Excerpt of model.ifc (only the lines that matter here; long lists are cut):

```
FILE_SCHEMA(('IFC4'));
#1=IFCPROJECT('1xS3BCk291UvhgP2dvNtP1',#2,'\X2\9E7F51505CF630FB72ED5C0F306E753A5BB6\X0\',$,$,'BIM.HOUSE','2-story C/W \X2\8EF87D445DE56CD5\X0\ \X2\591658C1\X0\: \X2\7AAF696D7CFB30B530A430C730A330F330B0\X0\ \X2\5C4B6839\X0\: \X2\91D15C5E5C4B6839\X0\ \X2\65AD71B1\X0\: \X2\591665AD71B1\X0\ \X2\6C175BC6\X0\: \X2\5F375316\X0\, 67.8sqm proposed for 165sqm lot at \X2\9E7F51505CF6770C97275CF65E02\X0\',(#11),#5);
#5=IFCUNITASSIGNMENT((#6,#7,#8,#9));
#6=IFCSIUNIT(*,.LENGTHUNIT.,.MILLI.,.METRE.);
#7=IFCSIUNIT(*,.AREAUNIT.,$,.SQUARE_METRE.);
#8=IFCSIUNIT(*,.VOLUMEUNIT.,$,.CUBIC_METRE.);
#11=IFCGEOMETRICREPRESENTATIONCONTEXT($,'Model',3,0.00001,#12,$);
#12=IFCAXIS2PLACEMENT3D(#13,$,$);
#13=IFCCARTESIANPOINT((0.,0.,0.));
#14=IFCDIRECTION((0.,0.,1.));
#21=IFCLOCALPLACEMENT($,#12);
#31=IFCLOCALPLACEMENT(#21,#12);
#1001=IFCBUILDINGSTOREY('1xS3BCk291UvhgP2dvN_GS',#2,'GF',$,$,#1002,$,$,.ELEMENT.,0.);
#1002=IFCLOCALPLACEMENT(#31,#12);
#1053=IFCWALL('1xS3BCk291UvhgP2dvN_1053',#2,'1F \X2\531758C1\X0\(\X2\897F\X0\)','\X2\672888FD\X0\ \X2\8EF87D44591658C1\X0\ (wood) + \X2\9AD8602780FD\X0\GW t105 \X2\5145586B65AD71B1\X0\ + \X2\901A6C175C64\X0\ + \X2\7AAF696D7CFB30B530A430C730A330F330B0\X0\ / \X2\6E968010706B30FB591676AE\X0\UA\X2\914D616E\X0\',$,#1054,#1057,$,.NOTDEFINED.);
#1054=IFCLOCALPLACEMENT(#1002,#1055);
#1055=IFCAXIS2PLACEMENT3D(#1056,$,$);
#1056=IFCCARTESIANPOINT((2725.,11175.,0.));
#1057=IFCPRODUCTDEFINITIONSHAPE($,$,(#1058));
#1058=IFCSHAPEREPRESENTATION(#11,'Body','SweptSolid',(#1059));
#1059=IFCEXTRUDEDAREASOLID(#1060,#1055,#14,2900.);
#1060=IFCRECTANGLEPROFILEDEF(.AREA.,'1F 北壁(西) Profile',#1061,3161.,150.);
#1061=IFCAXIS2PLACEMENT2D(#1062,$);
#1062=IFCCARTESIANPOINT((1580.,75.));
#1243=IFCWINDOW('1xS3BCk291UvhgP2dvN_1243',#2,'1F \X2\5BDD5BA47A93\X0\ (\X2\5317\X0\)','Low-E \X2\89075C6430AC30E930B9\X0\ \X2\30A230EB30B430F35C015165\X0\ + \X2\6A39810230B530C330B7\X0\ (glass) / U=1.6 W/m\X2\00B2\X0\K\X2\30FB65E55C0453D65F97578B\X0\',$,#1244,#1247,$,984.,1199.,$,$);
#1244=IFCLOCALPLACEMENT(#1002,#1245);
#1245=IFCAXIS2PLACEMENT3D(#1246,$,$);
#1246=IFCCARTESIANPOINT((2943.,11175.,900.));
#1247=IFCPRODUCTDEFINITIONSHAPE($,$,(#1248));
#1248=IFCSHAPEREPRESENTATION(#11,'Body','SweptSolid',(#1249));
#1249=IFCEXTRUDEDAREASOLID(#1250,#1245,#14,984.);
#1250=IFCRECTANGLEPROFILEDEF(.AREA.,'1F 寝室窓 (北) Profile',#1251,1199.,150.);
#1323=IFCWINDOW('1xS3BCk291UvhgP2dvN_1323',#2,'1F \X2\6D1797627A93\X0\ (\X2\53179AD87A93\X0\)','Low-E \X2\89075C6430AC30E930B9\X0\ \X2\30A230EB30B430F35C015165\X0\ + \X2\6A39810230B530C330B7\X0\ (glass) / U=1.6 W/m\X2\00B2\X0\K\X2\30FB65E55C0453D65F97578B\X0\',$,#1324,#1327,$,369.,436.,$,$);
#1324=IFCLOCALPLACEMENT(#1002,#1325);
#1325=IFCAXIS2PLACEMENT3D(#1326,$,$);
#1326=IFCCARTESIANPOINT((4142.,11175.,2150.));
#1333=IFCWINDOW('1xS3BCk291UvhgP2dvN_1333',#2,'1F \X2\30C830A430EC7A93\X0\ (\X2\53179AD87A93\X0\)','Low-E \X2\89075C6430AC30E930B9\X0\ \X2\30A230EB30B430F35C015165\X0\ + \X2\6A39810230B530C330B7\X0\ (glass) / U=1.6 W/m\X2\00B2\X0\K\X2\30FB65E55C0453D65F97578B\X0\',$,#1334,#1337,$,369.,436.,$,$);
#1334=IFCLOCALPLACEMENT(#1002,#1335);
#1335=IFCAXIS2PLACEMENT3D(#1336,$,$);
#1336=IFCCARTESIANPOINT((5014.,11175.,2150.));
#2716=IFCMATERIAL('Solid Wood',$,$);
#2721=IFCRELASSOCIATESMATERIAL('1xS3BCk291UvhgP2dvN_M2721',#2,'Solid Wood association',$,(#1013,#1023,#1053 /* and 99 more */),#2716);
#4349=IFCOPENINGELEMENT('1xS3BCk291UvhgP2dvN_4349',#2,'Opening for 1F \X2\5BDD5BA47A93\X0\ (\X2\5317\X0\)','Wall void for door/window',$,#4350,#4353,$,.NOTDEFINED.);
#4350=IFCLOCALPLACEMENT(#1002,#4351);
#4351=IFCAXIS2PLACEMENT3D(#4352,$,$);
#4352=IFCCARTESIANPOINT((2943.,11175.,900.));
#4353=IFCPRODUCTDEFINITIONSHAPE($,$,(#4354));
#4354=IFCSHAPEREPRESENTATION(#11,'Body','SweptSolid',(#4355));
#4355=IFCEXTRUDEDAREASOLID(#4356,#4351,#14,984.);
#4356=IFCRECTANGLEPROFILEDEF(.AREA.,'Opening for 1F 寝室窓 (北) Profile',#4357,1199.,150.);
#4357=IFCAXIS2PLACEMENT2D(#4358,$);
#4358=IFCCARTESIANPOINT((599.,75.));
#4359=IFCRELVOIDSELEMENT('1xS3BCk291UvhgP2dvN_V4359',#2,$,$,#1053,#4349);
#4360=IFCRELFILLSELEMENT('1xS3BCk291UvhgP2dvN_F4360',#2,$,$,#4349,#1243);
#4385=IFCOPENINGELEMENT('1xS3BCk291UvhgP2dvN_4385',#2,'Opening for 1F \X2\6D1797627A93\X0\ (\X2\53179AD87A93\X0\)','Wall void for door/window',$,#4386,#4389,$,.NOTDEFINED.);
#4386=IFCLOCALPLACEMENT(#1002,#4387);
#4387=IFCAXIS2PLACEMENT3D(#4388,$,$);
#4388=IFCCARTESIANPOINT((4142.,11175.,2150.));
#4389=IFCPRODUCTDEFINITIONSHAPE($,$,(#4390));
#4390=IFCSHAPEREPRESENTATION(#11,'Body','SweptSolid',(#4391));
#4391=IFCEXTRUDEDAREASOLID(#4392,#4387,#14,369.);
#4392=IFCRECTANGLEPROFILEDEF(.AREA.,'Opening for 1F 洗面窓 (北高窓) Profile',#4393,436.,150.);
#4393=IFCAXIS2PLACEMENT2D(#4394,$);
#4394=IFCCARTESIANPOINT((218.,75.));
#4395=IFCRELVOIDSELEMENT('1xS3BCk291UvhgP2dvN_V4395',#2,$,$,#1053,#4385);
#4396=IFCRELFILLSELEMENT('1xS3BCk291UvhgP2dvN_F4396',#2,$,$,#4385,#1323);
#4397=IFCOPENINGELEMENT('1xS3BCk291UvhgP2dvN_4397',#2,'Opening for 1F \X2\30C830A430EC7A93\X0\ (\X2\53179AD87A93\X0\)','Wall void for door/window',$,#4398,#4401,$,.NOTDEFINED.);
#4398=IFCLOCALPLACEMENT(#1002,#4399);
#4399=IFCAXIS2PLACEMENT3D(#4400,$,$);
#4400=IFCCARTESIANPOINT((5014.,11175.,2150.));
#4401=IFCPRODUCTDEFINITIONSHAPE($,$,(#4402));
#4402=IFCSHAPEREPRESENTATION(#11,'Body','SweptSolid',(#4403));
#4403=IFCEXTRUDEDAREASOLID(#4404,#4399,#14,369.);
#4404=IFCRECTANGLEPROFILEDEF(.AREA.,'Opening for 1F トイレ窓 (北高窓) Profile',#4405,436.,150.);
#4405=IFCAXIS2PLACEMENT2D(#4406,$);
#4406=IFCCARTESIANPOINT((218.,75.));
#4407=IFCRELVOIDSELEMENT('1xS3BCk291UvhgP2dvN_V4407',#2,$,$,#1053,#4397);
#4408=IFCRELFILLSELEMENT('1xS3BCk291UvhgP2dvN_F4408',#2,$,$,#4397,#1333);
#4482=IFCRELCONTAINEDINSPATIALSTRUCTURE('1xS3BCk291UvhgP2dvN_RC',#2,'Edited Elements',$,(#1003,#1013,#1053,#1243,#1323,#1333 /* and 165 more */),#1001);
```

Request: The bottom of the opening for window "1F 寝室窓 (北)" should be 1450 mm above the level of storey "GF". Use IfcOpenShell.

```python
import numpy as np
import ifcopenshell
import ifcopenshell.api.geometry
import ifcopenshell.geom
import ifcopenshell.util.element
import ifcopenshell.util.placement
import ifcopenshell.util.shape
import ifcopenshell.util.unit

model = ifcopenshell.open("model.ifc")
unit_scale = ifcopenshell.util.unit.calculate_unit_scale(model)

window = model.by_guid("1xS3BCk291UvhgP2dvN_1243")
opening = window.FillsVoids[0].RelatingOpeningElement
storey = ifcopenshell.util.element.get_container(window, ifc_class="IfcBuildingStorey")
level = ifcopenshell.util.placement.get_local_placement(storey.ObjectPlacement)[2, 3]

# The opening's origin need not be at the sill, so measure its lowest point.
shape = ifcopenshell.geom.create_shape(ifcopenshell.geom.settings(), opening)
bottom = ifcopenshell.util.shape.get_shape_bottom_elevation(shape, shape.geometry) / unit_scale
dz = level + 1.45 / unit_scale - bottom

shift = np.array([0.0, 0.0, dz])
# The window is not placed relative to its opening, so move both.
for product in (opening, window):
    matrix = ifcopenshell.util.placement.get_local_placement(product.ObjectPlacement)
    matrix[:3, 3] += shift
    ifcopenshell.api.geometry.edit_object_placement(model, product=product, matrix=matrix, is_si=False)

print(f"moved by {dz * unit_scale:+.3f} m")

model.write("model_rev.ifc")
```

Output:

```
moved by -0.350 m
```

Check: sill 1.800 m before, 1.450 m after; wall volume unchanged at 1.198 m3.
